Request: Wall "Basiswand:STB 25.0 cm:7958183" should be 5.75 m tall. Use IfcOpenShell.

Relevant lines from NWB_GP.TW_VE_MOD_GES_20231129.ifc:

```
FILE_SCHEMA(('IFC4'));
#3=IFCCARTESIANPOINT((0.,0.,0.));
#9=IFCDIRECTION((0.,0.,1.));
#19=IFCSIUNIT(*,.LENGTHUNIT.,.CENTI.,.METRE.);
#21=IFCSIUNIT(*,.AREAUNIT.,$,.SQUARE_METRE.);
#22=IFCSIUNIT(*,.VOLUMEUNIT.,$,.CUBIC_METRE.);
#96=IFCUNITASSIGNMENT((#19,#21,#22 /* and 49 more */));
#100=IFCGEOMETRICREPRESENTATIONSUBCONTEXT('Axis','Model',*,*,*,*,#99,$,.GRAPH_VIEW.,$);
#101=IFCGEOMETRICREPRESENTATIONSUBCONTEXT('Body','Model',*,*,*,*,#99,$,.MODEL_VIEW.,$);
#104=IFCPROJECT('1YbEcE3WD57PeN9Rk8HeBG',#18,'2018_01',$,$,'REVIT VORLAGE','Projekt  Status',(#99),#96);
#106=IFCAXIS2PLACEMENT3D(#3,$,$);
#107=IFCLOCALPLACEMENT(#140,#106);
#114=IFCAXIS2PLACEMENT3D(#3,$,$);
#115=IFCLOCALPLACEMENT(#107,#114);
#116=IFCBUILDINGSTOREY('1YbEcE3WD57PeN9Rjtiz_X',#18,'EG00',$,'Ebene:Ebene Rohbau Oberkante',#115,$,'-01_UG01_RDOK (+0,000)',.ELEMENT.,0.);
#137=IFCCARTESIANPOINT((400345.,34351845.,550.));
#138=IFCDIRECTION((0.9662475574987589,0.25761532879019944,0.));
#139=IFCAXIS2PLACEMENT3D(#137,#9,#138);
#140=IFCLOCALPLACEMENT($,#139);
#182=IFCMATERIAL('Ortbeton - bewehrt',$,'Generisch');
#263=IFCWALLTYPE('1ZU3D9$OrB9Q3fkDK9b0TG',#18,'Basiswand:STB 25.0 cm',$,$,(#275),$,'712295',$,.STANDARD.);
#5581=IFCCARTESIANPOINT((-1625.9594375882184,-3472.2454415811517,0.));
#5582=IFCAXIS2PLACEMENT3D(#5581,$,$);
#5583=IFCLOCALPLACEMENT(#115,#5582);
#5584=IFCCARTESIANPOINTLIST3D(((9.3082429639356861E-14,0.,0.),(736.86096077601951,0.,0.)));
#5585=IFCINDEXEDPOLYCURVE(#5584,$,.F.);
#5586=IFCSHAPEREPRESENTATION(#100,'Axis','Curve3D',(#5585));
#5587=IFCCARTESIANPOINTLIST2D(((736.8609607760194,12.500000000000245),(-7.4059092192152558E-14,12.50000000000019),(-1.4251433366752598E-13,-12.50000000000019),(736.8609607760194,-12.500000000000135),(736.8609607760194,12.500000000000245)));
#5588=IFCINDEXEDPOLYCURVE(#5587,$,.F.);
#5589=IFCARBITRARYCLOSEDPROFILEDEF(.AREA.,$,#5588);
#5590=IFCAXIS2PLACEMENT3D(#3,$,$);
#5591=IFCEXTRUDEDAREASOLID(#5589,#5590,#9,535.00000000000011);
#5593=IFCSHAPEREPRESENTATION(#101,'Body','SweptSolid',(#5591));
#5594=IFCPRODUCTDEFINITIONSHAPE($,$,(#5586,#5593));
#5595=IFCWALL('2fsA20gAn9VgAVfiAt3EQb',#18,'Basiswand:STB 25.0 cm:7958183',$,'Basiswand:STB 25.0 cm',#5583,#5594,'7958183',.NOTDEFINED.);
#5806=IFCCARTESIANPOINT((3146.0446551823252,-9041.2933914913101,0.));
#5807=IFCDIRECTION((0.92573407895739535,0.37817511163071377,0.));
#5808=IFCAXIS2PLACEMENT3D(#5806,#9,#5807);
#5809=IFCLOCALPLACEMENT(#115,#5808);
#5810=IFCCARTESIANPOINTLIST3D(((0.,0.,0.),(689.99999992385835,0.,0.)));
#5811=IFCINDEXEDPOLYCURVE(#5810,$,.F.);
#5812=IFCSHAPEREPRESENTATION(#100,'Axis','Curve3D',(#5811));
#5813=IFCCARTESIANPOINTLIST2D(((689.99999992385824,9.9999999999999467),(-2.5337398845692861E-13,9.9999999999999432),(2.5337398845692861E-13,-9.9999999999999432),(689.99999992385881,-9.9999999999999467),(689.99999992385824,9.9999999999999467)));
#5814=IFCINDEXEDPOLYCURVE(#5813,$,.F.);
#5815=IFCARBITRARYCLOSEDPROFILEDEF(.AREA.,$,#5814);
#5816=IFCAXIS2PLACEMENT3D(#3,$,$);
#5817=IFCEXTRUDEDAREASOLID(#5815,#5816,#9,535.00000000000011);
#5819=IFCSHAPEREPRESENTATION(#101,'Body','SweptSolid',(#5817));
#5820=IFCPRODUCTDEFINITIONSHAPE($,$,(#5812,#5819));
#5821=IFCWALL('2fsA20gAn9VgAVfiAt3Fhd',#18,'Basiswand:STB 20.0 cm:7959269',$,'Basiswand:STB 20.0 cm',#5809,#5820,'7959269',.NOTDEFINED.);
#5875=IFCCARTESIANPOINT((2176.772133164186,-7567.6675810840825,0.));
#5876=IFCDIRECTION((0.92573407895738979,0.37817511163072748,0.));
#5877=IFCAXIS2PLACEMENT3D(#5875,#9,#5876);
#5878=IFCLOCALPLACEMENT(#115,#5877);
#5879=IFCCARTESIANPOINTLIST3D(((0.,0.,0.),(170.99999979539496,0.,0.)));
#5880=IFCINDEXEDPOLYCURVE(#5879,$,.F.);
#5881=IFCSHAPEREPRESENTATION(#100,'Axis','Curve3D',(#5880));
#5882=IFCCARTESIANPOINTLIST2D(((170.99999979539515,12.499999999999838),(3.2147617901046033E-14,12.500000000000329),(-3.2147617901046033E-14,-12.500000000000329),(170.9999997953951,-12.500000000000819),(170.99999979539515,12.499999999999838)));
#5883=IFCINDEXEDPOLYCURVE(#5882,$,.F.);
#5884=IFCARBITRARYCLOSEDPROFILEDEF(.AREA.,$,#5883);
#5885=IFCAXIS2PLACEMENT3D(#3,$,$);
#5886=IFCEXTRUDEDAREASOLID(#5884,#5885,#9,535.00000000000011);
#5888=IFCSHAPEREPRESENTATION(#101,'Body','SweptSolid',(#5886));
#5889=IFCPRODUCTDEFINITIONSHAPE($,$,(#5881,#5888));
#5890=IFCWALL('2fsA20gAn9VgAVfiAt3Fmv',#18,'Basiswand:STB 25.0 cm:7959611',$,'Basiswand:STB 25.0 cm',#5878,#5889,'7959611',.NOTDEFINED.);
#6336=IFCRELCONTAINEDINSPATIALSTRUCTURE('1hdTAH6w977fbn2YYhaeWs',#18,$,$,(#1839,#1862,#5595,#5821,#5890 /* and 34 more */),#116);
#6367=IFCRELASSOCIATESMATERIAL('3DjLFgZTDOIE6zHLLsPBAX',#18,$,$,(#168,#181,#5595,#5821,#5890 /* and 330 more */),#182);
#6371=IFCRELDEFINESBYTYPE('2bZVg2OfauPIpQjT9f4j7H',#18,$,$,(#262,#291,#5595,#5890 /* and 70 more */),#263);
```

```python
import ifcopenshell
import ifcopenshell.geom
import ifcopenshell.util.representation
import ifcopenshell.util.shape
import ifcopenshell.util.unit

model = ifcopenshell.open("NWB_GP.TW_VE_MOD_GES_20231129.ifc")
unit_scale = ifcopenshell.util.unit.calculate_unit_scale(model)
settings = ifcopenshell.geom.settings()


def volume(element):
    """Net volume in cubic metres, openings subtracted."""
    shape = ifcopenshell.geom.create_shape(settings, element)
    return ifcopenshell.util.shape.get_volume(shape.geometry)


wall = model.by_guid("2fsA20gAn9VgAVfiAt3EQb")
before = volume(wall)

body = ifcopenshell.util.representation.get_representation(wall, "Model", "Body")
solid = body.Items[0]
old_height = solid.Depth
solid.Depth = 5.75 / unit_scale
after = volume(wall)

print(f"height {old_height:g} -> {solid.Depth:g}, volume {before:.3f} -> {after:.3f} m3")

model.write("NWB_GP.TW_VE_MOD_GES_20231129_updated.ifc")
```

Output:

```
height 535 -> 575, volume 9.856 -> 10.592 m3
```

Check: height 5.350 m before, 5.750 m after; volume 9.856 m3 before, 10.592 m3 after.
